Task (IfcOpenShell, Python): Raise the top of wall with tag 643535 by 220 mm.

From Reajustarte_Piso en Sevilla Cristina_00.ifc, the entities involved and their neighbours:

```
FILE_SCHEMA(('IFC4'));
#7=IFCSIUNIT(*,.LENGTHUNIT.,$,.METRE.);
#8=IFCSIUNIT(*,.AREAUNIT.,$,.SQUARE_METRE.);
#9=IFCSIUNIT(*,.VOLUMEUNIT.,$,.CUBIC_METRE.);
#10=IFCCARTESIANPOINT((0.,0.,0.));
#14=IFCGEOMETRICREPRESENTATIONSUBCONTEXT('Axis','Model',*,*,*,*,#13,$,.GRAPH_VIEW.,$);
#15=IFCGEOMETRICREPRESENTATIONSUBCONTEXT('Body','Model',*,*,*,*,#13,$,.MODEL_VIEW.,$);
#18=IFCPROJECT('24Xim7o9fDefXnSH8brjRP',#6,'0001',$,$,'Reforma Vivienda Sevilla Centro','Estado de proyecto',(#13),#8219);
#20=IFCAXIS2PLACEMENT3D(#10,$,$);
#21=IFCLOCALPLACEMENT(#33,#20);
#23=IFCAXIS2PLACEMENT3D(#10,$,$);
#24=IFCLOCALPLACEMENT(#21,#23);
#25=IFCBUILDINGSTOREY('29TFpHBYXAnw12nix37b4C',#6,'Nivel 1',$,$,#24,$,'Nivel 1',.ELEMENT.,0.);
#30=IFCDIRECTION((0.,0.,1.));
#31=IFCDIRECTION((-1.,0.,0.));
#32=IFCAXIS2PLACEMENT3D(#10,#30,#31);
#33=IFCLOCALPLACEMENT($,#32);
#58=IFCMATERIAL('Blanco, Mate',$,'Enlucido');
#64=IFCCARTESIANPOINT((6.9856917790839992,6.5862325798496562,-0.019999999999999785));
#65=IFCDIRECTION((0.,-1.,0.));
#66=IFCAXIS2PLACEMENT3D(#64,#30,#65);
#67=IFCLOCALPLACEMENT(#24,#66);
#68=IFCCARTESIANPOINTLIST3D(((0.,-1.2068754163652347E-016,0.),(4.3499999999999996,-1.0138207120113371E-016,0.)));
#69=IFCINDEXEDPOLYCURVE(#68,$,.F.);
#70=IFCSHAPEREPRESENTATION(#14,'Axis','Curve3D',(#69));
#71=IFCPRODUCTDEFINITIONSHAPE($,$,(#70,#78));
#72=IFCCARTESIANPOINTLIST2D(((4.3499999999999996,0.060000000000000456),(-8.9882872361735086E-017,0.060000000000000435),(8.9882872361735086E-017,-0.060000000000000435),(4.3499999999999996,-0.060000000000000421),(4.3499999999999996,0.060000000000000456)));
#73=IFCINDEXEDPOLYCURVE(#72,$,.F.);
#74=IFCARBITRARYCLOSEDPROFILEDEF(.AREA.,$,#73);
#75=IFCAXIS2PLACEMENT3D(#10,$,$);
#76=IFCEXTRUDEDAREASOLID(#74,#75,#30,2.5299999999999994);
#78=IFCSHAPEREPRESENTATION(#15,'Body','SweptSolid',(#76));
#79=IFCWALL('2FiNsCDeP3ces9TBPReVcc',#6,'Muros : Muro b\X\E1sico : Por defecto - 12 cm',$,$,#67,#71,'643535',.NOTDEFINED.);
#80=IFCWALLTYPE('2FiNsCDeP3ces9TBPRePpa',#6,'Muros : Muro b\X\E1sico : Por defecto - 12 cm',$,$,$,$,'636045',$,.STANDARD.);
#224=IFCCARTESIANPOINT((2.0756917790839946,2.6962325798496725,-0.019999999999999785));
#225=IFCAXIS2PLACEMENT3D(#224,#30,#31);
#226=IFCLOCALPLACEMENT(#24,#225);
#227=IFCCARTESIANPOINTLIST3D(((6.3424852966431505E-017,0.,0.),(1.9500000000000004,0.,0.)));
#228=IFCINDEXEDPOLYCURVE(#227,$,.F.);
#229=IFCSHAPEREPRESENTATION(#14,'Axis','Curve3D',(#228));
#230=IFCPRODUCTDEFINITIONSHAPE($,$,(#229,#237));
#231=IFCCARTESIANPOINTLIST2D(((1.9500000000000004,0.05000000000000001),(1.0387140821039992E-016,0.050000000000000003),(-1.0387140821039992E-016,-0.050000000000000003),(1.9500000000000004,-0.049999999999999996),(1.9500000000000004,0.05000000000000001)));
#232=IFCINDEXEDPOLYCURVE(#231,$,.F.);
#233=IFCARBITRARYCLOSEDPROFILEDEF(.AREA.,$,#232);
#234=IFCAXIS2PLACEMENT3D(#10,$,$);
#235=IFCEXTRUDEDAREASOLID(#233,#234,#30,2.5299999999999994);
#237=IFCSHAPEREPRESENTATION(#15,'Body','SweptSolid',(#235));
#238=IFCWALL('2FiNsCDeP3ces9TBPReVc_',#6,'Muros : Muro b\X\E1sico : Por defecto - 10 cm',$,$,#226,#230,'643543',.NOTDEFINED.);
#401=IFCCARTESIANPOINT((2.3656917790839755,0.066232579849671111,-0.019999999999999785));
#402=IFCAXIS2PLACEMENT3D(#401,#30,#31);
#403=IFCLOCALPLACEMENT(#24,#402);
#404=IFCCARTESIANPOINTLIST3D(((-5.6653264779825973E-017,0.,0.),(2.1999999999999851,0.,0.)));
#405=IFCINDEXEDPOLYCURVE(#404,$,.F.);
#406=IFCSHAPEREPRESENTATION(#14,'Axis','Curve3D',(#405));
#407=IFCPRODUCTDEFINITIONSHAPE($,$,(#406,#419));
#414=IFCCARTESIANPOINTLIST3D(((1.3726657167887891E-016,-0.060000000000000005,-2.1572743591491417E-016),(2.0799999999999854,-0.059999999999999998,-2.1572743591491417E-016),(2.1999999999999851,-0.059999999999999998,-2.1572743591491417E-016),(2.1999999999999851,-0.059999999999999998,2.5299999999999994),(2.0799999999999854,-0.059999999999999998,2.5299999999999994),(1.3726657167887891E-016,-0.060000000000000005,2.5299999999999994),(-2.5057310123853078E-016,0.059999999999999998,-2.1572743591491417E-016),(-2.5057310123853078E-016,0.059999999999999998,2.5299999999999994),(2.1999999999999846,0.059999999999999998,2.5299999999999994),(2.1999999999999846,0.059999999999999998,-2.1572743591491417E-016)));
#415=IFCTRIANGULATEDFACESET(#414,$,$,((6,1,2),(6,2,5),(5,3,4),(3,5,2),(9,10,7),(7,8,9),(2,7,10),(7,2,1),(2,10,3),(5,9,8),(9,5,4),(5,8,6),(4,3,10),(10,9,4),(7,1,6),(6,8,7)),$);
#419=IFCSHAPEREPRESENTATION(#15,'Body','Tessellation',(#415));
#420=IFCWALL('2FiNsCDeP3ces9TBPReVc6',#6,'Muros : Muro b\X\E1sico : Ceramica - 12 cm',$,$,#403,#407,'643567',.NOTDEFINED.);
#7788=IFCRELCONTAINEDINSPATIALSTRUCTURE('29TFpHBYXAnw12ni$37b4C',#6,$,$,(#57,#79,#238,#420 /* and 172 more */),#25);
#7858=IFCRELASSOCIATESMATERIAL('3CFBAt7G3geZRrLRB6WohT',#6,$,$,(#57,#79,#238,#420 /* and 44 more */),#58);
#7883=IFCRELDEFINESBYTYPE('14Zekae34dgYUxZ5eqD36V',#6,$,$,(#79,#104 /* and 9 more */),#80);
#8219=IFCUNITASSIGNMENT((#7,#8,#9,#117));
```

```python
import ifcopenshell
import ifcopenshell.geom
import ifcopenshell.util.representation
import ifcopenshell.util.shape

model = ifcopenshell.open("Reajustarte_Piso en Sevilla Cristina_00.ifc")
settings = ifcopenshell.geom.settings()


def volume(element):
    """Net volume in cubic metres, openings subtracted."""
    shape = ifcopenshell.geom.create_shape(settings, element)
    return ifcopenshell.util.shape.get_volume(shape.geometry)


wall = model.by_guid("2FiNsCDeP3ces9TBPReVcc")
before = volume(wall)

body = ifcopenshell.util.representation.get_representation(wall, "Model", "Body")
solid = body.Items[0]
old_height = solid.Depth
solid.Depth += 0.22
after = volume(wall)

print(f"height {old_height:g} -> {solid.Depth:g}, volume {before:.3f} -> {after:.3f} m3")

model.write("Reajustarte_Piso en Sevilla Cristina_00_updated.ifc")
```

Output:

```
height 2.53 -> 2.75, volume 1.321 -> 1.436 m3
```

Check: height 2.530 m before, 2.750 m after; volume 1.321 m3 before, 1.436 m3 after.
